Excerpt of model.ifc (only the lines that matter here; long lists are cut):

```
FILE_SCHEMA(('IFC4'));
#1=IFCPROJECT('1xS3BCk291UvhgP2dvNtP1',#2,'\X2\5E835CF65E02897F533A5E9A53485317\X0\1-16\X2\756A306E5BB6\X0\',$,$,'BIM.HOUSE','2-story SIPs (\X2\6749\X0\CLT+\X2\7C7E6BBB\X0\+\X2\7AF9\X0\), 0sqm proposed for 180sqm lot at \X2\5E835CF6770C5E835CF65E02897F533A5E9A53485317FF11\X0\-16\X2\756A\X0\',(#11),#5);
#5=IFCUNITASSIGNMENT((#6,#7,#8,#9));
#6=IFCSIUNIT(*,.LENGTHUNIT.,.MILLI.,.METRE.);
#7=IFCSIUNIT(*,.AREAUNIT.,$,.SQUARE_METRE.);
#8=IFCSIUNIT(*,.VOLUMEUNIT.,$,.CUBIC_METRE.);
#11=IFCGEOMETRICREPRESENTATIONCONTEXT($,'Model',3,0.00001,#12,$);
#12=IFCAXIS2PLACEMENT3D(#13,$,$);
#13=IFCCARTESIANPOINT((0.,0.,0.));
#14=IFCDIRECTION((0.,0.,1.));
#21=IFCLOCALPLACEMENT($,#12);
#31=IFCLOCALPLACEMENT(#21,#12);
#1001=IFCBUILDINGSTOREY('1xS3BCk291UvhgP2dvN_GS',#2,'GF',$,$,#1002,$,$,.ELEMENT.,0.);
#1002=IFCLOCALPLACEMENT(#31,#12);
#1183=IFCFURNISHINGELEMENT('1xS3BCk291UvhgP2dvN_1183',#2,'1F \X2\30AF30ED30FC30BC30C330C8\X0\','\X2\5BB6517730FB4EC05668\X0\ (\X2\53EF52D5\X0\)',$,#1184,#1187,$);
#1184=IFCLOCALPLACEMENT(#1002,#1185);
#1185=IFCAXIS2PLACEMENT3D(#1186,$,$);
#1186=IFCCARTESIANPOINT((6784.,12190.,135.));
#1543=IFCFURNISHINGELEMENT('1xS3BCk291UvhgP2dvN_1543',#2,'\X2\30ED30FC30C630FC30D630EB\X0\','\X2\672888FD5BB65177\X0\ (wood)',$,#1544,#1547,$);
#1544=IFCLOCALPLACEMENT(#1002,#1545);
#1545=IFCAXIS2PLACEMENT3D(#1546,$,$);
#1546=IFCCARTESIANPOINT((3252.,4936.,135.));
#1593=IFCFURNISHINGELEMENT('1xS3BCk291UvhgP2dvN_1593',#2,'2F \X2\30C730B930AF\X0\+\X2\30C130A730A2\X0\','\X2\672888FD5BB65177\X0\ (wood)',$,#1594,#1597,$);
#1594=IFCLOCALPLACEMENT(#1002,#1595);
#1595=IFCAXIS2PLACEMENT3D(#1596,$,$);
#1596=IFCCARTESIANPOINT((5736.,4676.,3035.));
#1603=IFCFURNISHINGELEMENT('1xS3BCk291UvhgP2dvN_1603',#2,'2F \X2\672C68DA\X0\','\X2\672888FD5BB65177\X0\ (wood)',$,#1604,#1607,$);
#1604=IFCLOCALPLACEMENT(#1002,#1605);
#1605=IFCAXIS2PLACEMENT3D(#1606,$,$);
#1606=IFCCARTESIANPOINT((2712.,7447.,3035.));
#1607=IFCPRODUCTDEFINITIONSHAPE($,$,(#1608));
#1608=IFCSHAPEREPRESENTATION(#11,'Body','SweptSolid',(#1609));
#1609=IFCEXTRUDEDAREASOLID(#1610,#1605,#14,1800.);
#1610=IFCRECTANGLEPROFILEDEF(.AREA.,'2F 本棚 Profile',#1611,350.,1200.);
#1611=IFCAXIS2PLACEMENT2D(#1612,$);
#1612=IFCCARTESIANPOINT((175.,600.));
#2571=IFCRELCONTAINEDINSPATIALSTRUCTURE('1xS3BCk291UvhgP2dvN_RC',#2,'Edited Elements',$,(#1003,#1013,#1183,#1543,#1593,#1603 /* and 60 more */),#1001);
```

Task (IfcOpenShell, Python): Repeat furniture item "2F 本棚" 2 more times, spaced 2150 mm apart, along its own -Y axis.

```python
import ifcopenshell
import ifcopenshell.api.geometry
import ifcopenshell.api.root
import ifcopenshell.util.element
import ifcopenshell.util.placement

model = ifcopenshell.open("model.ifc")


def reuse_history(source, copy):
    """copy_class also copies each property set's owner history, people and application; keep the originals."""
    for rel in copy.IsDefinedBy:
        if rel.is_a("IfcRelDefinesByProperties") and (history := rel.RelatingPropertyDefinition.OwnerHistory):
            rel.RelatingPropertyDefinition.OwnerHistory = source.OwnerHistory
            ifcopenshell.util.element.remove_deep2(model, history)


source = model.by_guid("1xS3BCk291UvhgP2dvN_1603")
base = ifcopenshell.util.placement.get_local_placement(source.ObjectPlacement)
step = -base[:3, 1] * 2150.0

for i in range(1, 3):
    copy = ifcopenshell.api.root.copy_class(model, product=source)
    copy.Representation = ifcopenshell.util.element.copy_deep(
        model, source.Representation, exclude=["IfcGeometricRepresentationContext", "IfcRepresentationMap"]
    )
    reuse_history(source, copy)
    matrix = base.copy()
    matrix[:3, 3] += i * step
    print("added at", matrix[:3, 3].round(3) + 0.0)
    ifcopenshell.api.geometry.edit_object_placement(model, product=copy, matrix=matrix, is_si=False)

model.write("model_v2.ifc")
```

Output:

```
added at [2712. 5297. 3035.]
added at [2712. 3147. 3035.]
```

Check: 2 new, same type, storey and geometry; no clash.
